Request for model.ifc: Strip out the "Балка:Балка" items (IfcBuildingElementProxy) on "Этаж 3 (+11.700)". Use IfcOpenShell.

First a look at what the model holds.

```python
import ifcopenshell
import ifcopenshell.util.element

model = ifcopenshell.open("model.ifc")
print(model.schema)
storey = next(s for s in model.by_type("IfcBuildingStorey") if s.Name == "Этаж 3 (+11.700)")
proxies = [e for e in ifcopenshell.util.element.get_decomposition(storey) if e.is_a("IfcBuildingElementProxy")]
seen = {}
for e in proxies:
    element_type = ifcopenshell.util.element.get_type(e)
    name = element_type.Name if element_type not in (None, e) else None
    seen[name] = seen.get(name, 0) + 1
for name, count in sorted(seen.items(), key=str):
    print(count, "x", name)
```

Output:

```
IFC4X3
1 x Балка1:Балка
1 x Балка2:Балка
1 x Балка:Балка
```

```python
import ifcopenshell
import ifcopenshell.api.root
import ifcopenshell.util.element

model = ifcopenshell.open("model.ifc")

storey = next(s for s in model.by_type("IfcBuildingStorey") if s.Name == "Этаж 3 (+11.700)")
proxies = [e for e in ifcopenshell.util.element.get_decomposition(storey) if e.is_a("IfcBuildingElementProxy")]
targets = [e for e in proxies if (t := ifcopenshell.util.element.get_type(e)) not in (None, e) and t.Name == "Балка:Балка"]

for e in targets:
    ifcopenshell.api.root.remove_product(model, product=e)
print(len(targets), "removed")

model.write("model_v2.ifc")
```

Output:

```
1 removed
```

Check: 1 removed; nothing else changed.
